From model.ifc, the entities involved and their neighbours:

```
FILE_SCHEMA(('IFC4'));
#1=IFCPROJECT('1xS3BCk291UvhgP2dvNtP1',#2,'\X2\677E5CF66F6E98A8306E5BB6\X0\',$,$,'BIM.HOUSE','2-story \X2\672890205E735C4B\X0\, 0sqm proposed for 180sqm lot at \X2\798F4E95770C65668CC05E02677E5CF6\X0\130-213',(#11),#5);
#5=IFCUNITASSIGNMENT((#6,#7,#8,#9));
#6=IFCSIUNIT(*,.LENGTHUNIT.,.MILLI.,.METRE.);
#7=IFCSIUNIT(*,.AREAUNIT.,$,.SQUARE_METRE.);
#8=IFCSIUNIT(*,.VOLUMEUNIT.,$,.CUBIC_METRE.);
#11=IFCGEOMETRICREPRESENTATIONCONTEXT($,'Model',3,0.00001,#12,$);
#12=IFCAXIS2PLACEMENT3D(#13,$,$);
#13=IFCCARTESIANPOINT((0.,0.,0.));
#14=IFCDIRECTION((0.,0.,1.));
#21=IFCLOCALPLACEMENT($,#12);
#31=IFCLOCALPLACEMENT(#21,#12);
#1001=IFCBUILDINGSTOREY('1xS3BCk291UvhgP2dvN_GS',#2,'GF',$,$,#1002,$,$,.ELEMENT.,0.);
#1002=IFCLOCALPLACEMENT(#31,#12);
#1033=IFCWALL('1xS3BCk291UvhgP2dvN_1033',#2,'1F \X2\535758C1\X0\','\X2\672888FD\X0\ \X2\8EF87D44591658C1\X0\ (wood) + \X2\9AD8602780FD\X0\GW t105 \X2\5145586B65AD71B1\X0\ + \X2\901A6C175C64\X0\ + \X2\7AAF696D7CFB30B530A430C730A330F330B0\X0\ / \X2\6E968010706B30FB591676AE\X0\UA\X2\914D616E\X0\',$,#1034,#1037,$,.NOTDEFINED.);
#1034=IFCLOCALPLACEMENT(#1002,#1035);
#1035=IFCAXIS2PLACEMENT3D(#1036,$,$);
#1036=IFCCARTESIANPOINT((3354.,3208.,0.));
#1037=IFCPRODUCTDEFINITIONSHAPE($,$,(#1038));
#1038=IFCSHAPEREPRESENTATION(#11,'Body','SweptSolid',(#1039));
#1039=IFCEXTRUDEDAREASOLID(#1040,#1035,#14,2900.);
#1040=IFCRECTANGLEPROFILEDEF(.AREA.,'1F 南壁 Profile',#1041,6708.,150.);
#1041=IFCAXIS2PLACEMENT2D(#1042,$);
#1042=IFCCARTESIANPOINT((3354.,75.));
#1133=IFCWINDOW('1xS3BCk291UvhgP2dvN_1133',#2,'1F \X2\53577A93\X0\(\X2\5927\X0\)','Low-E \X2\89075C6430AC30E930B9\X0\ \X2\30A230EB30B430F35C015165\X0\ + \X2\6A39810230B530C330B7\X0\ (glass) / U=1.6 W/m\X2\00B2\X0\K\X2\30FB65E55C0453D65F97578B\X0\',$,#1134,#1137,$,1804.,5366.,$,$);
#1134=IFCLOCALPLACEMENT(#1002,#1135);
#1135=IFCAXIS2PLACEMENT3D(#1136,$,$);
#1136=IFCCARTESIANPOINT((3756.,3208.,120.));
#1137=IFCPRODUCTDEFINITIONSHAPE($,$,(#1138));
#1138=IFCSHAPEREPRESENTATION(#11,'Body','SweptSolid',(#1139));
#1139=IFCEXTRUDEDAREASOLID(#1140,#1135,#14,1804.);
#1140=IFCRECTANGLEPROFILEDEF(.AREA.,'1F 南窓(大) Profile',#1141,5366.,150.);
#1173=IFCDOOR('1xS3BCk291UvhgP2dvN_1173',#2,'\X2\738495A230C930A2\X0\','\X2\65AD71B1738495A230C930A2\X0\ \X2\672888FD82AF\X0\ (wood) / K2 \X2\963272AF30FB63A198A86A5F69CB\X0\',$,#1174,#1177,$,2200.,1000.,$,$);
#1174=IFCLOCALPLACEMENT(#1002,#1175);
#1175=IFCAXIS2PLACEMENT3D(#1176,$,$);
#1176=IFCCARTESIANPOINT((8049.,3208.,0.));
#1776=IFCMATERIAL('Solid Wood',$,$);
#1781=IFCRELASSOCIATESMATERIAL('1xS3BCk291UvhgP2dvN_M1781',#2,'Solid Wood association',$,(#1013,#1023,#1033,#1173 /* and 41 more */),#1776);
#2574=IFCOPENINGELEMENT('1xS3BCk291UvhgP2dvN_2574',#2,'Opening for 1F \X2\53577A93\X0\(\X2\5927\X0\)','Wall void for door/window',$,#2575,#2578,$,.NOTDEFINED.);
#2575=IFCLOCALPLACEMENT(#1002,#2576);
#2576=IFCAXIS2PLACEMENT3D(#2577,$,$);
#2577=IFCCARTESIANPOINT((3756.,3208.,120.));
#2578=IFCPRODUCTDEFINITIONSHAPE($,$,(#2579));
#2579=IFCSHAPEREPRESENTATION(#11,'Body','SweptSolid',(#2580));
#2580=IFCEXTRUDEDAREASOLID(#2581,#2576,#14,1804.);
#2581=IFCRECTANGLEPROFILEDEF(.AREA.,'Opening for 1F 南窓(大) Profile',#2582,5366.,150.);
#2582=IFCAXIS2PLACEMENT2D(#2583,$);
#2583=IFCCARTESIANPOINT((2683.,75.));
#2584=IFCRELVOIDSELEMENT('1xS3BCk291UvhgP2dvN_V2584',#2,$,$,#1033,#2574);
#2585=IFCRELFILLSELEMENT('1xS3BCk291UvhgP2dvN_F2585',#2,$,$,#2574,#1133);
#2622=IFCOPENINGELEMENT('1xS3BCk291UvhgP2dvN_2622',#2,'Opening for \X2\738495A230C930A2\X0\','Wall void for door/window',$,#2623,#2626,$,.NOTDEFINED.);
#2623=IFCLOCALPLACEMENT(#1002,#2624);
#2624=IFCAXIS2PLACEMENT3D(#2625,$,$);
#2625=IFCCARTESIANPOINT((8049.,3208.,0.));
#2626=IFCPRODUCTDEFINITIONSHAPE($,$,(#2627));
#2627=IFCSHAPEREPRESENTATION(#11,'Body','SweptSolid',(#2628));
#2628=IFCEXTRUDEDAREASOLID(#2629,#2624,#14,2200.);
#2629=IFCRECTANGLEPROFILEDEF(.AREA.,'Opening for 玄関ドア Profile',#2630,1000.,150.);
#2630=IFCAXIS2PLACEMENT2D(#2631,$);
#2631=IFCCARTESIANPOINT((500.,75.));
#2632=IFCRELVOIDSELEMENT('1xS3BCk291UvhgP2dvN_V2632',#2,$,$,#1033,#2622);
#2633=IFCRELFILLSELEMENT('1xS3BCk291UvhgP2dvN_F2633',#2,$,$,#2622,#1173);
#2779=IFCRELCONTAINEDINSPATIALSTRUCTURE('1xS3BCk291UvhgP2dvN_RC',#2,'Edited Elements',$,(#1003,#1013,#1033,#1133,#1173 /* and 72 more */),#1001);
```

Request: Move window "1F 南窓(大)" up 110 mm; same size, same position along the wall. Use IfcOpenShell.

```python
import numpy as np
import ifcopenshell
import ifcopenshell.api.geometry
import ifcopenshell.util.placement
import ifcopenshell.util.unit

model = ifcopenshell.open("model.ifc")
unit_scale = ifcopenshell.util.unit.calculate_unit_scale(model)

window = model.by_guid("1xS3BCk291UvhgP2dvN_1133")
opening = window.FillsVoids[0].RelatingOpeningElement
dz = 0.11 / unit_scale

shift = np.array([0.0, 0.0, dz])
# The window is not placed relative to its opening, so move both.
for product in (opening, window):
    matrix = ifcopenshell.util.placement.get_local_placement(product.ObjectPlacement)
    matrix[:3, 3] += shift
    ifcopenshell.api.geometry.edit_object_placement(model, product=product, matrix=matrix, is_si=False)

print(f"moved by {dz * unit_scale:+.3f} m")

model.write("model_v2.ifc")
```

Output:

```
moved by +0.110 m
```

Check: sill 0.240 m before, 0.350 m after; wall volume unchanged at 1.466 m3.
